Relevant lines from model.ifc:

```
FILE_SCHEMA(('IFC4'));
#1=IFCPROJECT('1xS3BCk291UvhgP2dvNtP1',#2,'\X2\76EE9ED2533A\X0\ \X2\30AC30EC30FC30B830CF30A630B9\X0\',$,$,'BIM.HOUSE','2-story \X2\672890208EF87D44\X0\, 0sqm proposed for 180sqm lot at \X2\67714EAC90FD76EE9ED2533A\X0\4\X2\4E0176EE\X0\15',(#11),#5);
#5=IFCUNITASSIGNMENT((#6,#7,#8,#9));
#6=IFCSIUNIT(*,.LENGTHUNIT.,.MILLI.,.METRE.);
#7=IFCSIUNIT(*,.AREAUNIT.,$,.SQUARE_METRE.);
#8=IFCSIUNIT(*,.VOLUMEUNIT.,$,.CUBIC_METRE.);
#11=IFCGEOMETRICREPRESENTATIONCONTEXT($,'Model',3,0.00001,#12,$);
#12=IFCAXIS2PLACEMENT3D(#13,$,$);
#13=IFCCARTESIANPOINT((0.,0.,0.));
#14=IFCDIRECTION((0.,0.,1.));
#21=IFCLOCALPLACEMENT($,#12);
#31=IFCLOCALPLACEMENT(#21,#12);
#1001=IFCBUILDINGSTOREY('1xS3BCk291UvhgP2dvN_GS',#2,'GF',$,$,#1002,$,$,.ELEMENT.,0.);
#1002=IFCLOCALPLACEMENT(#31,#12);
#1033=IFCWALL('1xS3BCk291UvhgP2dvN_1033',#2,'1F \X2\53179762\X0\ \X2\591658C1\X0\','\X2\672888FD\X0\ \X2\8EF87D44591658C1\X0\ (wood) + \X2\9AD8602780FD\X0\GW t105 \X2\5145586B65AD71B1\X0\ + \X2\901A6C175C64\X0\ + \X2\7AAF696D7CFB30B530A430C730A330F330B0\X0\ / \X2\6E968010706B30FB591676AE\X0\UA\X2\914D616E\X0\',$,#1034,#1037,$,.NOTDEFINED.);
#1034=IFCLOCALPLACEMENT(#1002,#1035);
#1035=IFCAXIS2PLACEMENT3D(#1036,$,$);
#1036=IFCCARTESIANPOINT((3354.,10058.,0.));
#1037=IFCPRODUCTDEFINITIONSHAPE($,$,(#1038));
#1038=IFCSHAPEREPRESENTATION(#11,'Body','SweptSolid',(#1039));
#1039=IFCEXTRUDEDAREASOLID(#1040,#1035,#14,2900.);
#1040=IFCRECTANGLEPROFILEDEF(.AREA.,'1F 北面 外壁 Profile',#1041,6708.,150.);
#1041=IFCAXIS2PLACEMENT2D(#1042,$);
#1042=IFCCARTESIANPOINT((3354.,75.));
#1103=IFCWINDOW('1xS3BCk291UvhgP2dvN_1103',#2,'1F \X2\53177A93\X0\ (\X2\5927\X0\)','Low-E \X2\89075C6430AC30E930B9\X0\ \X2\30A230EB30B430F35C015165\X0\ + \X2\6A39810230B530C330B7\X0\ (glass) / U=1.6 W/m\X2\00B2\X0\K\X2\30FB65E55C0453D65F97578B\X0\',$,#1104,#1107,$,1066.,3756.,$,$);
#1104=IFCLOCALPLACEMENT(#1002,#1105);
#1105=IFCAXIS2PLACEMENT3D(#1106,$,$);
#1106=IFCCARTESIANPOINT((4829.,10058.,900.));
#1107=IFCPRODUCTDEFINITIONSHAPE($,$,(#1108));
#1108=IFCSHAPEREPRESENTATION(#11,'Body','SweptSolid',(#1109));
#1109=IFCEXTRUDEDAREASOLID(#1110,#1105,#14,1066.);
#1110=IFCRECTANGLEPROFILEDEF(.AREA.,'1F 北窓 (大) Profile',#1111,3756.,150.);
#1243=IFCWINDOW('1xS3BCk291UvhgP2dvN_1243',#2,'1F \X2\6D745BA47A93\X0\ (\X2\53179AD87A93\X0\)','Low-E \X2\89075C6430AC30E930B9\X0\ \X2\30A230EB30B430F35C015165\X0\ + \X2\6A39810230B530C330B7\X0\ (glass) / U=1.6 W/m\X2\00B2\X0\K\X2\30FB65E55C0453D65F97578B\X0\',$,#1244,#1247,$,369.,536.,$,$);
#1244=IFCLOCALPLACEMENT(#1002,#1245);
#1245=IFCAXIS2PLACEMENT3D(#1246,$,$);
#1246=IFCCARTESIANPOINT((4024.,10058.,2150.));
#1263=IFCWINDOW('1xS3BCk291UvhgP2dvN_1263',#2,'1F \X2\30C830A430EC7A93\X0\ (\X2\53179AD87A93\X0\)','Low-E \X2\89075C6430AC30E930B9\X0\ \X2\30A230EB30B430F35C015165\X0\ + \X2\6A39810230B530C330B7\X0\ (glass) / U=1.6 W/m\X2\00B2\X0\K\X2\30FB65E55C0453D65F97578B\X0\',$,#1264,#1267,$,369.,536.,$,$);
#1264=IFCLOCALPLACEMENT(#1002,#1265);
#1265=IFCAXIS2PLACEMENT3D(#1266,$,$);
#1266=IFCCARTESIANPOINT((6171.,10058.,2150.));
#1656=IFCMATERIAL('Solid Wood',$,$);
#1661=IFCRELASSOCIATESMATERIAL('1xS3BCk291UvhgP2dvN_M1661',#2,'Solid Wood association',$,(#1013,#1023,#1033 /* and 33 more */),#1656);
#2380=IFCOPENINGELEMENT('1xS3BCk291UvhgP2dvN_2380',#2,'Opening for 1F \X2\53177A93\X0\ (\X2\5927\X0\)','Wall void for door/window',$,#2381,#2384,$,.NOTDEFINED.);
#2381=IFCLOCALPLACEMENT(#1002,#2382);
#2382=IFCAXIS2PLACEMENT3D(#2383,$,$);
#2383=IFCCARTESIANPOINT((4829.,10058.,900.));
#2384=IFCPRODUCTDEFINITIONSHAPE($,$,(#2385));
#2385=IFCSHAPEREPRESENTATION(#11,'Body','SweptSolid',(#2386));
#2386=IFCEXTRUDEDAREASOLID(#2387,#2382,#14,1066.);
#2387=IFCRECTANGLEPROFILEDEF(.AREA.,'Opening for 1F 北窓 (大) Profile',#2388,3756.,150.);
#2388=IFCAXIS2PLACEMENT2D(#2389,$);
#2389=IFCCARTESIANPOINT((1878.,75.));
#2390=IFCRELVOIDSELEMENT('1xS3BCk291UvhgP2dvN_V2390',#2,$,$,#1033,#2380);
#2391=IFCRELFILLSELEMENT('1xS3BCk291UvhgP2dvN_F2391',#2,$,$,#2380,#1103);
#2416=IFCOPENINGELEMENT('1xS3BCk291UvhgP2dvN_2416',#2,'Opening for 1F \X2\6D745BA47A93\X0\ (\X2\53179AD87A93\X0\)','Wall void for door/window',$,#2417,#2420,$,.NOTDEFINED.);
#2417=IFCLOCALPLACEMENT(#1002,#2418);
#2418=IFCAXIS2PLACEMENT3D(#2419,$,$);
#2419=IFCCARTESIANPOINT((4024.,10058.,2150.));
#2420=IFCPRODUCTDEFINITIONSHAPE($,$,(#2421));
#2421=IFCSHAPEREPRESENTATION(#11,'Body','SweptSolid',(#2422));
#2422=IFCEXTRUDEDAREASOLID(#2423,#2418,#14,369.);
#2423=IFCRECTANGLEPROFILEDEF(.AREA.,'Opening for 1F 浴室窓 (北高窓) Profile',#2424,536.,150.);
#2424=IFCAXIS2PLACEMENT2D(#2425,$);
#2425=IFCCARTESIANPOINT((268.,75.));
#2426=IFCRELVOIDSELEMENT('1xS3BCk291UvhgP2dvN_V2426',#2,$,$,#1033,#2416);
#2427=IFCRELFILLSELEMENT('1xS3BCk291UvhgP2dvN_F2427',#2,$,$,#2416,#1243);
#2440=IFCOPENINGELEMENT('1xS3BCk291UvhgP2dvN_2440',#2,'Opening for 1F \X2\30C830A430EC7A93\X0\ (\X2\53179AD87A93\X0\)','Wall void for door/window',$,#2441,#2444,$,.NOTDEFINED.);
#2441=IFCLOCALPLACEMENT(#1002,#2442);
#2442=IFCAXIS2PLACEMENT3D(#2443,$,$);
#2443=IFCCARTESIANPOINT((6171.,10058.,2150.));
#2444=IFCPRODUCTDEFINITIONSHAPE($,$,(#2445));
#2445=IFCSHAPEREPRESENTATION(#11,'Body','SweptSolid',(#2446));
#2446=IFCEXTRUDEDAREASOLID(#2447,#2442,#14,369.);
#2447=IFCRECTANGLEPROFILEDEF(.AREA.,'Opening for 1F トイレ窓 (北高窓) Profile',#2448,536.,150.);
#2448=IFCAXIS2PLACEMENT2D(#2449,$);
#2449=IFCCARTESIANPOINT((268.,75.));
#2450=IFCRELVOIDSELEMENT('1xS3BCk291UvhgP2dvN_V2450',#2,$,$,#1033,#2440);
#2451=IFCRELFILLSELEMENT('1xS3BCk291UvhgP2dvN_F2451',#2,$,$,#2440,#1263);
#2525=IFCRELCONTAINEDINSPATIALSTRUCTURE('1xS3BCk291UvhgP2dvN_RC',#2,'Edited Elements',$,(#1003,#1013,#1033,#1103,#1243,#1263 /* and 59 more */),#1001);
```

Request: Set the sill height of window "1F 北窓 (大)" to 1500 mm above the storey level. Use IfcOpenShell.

```python
import numpy as np
import ifcopenshell
import ifcopenshell.api.geometry
import ifcopenshell.geom
import ifcopenshell.util.element
import ifcopenshell.util.placement
import ifcopenshell.util.shape
import ifcopenshell.util.unit

model = ifcopenshell.open("model.ifc")
unit_scale = ifcopenshell.util.unit.calculate_unit_scale(model)

window = model.by_id(1103)
opening = window.FillsVoids[0].RelatingOpeningElement
storey = ifcopenshell.util.element.get_container(window, ifc_class="IfcBuildingStorey")
level = ifcopenshell.util.placement.get_local_placement(storey.ObjectPlacement)[2, 3]

# The opening's origin need not be at the sill, so measure its lowest point.
shape = ifcopenshell.geom.create_shape(ifcopenshell.geom.settings(), opening)
bottom = ifcopenshell.util.shape.get_shape_bottom_elevation(shape, shape.geometry) / unit_scale
dz = level + 1500.0 - bottom

shift = np.array([0.0, 0.0, dz])
# The window is not placed relative to its opening, so move both.
for product in (opening, window):
    matrix = ifcopenshell.util.placement.get_local_placement(product.ObjectPlacement)
    matrix[:3, 3] += shift
    ifcopenshell.api.geometry.edit_object_placement(model, product=product, matrix=matrix, is_si=False)

print(f"moved by {dz * unit_scale:+.3f} m")

model.write("model_rev.ifc")
```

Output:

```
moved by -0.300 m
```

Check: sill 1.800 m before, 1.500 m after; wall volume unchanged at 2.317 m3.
